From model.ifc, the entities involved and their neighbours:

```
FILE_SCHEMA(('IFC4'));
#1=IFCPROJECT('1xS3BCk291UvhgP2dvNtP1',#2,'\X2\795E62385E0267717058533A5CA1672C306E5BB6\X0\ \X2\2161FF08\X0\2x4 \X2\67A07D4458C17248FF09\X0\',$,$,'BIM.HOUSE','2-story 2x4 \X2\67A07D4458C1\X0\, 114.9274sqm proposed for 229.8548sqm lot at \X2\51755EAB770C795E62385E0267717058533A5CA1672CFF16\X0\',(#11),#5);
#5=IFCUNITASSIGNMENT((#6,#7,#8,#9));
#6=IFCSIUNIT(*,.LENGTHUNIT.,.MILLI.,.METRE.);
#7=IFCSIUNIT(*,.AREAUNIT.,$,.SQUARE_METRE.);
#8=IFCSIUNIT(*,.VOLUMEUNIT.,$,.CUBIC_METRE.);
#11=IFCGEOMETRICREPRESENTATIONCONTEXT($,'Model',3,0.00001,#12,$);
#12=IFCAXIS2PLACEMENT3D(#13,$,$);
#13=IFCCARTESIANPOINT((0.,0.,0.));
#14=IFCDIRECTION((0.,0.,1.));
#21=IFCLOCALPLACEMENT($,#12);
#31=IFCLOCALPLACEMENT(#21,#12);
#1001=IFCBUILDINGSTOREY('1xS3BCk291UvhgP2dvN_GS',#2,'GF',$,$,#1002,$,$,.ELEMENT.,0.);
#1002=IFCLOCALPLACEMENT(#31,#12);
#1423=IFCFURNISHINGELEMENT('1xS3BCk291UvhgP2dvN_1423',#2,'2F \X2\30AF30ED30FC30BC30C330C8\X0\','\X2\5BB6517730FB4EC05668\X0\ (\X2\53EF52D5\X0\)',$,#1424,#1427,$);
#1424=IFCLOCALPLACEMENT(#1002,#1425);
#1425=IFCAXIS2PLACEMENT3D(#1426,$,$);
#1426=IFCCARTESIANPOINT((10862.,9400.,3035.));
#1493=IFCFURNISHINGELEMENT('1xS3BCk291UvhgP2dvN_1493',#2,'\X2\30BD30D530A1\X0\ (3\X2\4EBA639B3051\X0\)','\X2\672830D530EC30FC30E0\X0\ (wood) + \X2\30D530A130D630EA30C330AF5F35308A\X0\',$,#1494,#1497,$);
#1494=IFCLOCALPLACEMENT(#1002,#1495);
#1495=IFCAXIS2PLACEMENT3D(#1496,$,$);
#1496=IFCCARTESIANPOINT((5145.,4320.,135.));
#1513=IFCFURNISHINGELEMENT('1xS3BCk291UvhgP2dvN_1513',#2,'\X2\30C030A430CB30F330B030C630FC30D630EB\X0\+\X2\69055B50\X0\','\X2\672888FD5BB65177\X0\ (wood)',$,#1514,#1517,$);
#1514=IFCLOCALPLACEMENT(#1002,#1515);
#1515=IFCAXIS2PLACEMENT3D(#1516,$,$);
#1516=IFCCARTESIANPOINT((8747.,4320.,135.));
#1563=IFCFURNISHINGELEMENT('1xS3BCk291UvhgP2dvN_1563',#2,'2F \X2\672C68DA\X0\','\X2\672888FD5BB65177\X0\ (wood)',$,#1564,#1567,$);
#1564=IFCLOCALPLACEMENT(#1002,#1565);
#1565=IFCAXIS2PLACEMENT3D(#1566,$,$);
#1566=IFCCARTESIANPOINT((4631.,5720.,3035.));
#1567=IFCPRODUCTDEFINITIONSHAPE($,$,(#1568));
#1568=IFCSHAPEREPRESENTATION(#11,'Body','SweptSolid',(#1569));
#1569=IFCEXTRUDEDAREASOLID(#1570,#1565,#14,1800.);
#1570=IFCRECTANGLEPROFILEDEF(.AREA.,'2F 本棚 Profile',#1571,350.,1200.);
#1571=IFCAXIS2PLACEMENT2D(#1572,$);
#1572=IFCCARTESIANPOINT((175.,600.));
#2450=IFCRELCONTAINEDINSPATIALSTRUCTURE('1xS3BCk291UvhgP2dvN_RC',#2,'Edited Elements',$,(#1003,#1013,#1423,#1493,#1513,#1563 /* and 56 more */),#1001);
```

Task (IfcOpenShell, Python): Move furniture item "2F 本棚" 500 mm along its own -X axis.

```python
import ifcopenshell
import ifcopenshell.api.geometry
import ifcopenshell.util.placement
import ifcopenshell.util.unit

model = ifcopenshell.open("model.ifc")
unit_scale = ifcopenshell.util.unit.calculate_unit_scale(model)

item = model.by_guid("1xS3BCk291UvhgP2dvN_1563")
matrix = ifcopenshell.util.placement.get_local_placement(item.ObjectPlacement)
matrix[:3, 3] -= matrix[:3, 0] * 0.5 / unit_scale
ifcopenshell.api.geometry.edit_object_placement(model, product=item, matrix=matrix, is_si=False)

print(ifcopenshell.util.placement.get_local_placement(item.ObjectPlacement).round(3) + 0.0)

model.write("model-out.ifc")
```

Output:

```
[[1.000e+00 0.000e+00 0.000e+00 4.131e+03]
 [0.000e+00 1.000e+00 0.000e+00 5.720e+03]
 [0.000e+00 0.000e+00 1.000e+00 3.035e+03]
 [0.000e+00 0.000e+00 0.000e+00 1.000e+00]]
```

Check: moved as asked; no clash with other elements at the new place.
